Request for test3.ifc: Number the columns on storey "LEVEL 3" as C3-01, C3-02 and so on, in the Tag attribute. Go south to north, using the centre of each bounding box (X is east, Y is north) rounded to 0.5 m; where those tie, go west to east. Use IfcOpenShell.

First a look at what the model holds.

```python
import ifcopenshell
import ifcopenshell.util.element
import ifcopenshell.util.placement

model = ifcopenshell.open("test3.ifc")
print(model.schema)
storey = next(s for s in model.by_type("IfcBuildingStorey") if s.Name == "LEVEL 3")
columns = [e for e in ifcopenshell.util.element.get_decomposition(storey) if e.is_a("IfcColumn")]
for e in sorted(columns, key=lambda e: e.id()):
    origin = ifcopenshell.util.placement.get_local_placement(e.ObjectPlacement)[:3, 3]
    print(e.id(), e.Tag, e.Name, origin.round(2) + 0.0, sep=" | ")
```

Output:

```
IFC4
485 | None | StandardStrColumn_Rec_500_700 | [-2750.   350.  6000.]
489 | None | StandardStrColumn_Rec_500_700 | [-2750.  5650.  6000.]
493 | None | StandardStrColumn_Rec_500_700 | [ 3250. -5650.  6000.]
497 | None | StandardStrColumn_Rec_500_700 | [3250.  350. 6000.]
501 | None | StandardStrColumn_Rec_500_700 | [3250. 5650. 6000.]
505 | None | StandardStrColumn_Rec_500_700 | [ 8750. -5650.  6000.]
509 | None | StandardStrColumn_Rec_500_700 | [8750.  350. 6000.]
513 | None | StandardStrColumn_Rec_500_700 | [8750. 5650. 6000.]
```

```python
import ifcopenshell
import ifcopenshell.geom
import ifcopenshell.util.element
import ifcopenshell.util.shape

model = ifcopenshell.open("test3.ifc")
settings = ifcopenshell.geom.settings()
settings.set("use-world-coords", True)


def centre(element):
    shape = ifcopenshell.geom.create_shape(settings, element)
    return ifcopenshell.util.shape.get_bbox_centroid(shape.geometry)


storey = next(s for s in model.by_type("IfcBuildingStorey") if s.Name == "LEVEL 3")
columns = [e for e in ifcopenshell.util.element.get_decomposition(storey) if e.is_a("IfcColumn")]

# Insertion points can sit at a corner or the storey origin, so sort by the geometry (in metres).
centres = {e: centre(e) for e in columns}
columns.sort(key=lambda e: (round(centres[e][1] / 0.5), centres[e][0]))

for i, e in enumerate(columns, start=1):
    number = f"C3-{i:02d}"
    e.Tag = number
    print(e.id(), number)

model.write("test3_rev.ifc")
```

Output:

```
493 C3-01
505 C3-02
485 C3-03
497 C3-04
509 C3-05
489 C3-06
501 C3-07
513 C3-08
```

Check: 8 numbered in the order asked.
